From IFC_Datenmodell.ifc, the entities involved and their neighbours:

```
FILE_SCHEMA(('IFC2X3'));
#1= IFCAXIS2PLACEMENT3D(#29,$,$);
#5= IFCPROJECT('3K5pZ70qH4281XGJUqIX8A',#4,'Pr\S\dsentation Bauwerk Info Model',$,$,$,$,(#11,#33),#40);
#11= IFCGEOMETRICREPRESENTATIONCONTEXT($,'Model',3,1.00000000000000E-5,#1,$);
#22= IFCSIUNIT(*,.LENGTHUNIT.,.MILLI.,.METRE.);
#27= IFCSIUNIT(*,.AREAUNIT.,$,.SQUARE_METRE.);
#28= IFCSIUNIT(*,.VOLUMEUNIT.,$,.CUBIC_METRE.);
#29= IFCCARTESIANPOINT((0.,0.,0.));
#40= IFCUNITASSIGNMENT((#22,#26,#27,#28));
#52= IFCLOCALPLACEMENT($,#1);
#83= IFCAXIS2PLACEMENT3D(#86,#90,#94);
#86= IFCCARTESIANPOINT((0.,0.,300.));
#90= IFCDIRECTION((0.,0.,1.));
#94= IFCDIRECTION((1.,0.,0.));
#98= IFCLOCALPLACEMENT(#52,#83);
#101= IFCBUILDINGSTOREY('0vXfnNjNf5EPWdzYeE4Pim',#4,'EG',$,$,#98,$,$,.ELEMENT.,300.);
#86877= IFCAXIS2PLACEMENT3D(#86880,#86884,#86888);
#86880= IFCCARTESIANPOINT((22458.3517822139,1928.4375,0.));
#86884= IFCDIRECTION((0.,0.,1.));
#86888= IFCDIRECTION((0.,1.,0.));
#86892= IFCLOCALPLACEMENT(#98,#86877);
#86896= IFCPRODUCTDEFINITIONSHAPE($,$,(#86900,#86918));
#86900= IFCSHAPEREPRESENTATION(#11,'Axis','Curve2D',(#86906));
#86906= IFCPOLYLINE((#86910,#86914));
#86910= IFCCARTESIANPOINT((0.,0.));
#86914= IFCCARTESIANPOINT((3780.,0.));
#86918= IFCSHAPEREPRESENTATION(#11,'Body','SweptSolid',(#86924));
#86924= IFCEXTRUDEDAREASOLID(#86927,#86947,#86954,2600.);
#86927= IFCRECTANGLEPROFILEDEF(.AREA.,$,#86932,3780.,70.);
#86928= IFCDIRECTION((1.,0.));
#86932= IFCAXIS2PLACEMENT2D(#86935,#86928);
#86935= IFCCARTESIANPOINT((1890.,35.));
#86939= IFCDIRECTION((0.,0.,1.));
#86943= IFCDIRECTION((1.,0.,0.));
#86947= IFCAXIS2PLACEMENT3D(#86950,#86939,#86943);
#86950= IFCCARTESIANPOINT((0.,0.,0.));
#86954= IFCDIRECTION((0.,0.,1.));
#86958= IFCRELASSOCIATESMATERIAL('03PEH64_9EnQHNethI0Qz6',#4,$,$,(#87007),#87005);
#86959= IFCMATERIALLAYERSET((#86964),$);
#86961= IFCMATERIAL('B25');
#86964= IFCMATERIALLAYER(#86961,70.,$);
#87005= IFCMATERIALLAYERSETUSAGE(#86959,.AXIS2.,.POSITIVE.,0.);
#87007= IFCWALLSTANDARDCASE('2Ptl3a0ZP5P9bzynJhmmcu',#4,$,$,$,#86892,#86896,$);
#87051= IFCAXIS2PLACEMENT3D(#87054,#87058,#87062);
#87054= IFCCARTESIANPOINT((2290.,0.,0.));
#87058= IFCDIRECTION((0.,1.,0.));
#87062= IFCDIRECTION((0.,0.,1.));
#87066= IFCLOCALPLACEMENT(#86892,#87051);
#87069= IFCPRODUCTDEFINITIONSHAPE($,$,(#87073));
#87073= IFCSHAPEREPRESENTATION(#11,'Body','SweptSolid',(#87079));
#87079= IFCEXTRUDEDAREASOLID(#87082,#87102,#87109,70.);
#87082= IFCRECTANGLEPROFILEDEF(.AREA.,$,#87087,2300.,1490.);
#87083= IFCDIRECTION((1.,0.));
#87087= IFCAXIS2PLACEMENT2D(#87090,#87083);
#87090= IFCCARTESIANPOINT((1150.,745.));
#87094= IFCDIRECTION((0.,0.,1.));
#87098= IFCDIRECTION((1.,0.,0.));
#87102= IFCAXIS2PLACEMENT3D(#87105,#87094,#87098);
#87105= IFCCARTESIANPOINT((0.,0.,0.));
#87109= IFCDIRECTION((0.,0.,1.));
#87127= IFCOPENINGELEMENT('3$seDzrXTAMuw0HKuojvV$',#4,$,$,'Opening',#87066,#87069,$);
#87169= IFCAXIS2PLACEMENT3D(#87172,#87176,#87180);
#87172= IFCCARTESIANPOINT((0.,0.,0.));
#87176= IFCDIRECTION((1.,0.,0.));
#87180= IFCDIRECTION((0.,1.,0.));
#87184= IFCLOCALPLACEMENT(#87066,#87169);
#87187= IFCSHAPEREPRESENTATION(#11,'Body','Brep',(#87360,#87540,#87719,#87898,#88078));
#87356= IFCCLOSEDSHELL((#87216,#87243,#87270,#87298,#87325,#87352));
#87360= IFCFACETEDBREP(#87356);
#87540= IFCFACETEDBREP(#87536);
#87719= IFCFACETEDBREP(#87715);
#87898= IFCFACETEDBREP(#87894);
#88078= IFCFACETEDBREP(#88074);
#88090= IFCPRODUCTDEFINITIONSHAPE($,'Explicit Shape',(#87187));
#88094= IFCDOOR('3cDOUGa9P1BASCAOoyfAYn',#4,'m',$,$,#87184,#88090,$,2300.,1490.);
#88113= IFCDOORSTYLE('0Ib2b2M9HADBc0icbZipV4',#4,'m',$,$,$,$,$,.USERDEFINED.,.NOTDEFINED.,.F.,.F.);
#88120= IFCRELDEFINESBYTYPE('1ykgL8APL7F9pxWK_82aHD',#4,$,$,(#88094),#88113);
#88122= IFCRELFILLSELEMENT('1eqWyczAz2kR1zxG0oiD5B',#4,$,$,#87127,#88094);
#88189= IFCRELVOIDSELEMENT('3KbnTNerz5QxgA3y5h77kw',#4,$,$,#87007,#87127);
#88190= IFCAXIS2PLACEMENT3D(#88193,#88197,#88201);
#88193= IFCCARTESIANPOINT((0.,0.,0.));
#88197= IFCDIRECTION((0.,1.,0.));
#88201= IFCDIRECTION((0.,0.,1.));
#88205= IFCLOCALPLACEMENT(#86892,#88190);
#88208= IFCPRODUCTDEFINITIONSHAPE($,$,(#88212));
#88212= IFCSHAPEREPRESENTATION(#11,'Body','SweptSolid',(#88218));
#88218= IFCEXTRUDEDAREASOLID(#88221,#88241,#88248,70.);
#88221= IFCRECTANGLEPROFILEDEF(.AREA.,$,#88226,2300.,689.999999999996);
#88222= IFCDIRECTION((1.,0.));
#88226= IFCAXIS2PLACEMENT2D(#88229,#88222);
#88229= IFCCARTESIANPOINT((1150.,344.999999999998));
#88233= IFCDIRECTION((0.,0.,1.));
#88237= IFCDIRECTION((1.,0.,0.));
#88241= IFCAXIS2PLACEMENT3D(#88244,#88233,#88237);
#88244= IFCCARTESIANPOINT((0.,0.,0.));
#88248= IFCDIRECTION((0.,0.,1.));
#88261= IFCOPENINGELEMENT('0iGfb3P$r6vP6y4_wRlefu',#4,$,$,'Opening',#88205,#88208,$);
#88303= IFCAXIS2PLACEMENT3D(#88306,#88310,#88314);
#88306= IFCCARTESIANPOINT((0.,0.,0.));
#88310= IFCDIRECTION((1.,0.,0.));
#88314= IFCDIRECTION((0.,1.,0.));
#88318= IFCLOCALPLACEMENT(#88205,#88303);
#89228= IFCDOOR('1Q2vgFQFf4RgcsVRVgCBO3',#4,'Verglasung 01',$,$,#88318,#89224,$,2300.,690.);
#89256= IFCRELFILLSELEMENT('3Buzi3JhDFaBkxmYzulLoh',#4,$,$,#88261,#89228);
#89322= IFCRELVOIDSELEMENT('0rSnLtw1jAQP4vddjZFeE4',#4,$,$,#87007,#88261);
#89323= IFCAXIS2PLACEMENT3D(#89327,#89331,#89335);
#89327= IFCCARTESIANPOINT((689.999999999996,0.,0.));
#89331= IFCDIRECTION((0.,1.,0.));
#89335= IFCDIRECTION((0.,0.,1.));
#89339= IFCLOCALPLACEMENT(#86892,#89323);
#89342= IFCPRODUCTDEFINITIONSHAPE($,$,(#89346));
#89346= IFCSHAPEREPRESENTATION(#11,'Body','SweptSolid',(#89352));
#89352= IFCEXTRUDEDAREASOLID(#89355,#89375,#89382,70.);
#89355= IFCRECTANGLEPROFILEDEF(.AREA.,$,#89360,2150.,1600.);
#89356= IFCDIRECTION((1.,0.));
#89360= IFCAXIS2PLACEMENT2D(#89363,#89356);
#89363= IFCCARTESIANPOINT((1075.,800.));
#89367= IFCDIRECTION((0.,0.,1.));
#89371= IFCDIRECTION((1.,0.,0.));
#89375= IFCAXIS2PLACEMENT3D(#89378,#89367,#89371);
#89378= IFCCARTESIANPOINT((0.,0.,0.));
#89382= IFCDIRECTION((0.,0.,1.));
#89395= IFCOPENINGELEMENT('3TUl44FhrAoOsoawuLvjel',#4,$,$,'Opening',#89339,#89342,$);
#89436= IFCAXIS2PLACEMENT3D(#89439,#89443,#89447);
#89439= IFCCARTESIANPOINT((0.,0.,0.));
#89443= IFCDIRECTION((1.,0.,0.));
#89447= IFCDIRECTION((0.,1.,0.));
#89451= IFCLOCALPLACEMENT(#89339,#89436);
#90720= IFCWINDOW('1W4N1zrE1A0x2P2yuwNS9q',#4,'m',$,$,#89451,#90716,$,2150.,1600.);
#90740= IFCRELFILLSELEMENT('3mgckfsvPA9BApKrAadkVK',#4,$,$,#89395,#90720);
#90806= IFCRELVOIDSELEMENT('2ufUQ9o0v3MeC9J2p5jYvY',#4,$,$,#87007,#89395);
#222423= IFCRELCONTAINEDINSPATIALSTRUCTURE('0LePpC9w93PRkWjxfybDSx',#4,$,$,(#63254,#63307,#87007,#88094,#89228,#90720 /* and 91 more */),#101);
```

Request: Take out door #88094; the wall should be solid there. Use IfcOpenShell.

```python
import ifcopenshell
import ifcopenshell.api.feature
import ifcopenshell.api.root
import ifcopenshell.geom
import ifcopenshell.util.shape

model = ifcopenshell.open("IFC_Datenmodell.ifc")
settings = ifcopenshell.geom.settings()


def volume(element):
    """Net volume in cubic metres, openings subtracted."""
    shape = ifcopenshell.geom.create_shape(settings, element)
    return ifcopenshell.util.shape.get_volume(shape.geometry)


door = model.by_guid("3cDOUGa9P1BASCAOoyfAYn")
opening = door.FillsVoids[0].RelatingOpeningElement
wall = opening.VoidsElements[0].RelatingBuildingElement
before = volume(wall)

ifcopenshell.api.root.remove_product(model, product=door)
ifcopenshell.api.feature.remove_feature(model, feature=opening)

after = volume(wall)

print(f"wall volume {before:.3f} -> {after:.3f} m3")

model.write("IFC_Datenmodell_v2.ifc")
```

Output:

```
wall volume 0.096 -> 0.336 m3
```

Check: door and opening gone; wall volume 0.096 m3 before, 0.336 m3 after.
